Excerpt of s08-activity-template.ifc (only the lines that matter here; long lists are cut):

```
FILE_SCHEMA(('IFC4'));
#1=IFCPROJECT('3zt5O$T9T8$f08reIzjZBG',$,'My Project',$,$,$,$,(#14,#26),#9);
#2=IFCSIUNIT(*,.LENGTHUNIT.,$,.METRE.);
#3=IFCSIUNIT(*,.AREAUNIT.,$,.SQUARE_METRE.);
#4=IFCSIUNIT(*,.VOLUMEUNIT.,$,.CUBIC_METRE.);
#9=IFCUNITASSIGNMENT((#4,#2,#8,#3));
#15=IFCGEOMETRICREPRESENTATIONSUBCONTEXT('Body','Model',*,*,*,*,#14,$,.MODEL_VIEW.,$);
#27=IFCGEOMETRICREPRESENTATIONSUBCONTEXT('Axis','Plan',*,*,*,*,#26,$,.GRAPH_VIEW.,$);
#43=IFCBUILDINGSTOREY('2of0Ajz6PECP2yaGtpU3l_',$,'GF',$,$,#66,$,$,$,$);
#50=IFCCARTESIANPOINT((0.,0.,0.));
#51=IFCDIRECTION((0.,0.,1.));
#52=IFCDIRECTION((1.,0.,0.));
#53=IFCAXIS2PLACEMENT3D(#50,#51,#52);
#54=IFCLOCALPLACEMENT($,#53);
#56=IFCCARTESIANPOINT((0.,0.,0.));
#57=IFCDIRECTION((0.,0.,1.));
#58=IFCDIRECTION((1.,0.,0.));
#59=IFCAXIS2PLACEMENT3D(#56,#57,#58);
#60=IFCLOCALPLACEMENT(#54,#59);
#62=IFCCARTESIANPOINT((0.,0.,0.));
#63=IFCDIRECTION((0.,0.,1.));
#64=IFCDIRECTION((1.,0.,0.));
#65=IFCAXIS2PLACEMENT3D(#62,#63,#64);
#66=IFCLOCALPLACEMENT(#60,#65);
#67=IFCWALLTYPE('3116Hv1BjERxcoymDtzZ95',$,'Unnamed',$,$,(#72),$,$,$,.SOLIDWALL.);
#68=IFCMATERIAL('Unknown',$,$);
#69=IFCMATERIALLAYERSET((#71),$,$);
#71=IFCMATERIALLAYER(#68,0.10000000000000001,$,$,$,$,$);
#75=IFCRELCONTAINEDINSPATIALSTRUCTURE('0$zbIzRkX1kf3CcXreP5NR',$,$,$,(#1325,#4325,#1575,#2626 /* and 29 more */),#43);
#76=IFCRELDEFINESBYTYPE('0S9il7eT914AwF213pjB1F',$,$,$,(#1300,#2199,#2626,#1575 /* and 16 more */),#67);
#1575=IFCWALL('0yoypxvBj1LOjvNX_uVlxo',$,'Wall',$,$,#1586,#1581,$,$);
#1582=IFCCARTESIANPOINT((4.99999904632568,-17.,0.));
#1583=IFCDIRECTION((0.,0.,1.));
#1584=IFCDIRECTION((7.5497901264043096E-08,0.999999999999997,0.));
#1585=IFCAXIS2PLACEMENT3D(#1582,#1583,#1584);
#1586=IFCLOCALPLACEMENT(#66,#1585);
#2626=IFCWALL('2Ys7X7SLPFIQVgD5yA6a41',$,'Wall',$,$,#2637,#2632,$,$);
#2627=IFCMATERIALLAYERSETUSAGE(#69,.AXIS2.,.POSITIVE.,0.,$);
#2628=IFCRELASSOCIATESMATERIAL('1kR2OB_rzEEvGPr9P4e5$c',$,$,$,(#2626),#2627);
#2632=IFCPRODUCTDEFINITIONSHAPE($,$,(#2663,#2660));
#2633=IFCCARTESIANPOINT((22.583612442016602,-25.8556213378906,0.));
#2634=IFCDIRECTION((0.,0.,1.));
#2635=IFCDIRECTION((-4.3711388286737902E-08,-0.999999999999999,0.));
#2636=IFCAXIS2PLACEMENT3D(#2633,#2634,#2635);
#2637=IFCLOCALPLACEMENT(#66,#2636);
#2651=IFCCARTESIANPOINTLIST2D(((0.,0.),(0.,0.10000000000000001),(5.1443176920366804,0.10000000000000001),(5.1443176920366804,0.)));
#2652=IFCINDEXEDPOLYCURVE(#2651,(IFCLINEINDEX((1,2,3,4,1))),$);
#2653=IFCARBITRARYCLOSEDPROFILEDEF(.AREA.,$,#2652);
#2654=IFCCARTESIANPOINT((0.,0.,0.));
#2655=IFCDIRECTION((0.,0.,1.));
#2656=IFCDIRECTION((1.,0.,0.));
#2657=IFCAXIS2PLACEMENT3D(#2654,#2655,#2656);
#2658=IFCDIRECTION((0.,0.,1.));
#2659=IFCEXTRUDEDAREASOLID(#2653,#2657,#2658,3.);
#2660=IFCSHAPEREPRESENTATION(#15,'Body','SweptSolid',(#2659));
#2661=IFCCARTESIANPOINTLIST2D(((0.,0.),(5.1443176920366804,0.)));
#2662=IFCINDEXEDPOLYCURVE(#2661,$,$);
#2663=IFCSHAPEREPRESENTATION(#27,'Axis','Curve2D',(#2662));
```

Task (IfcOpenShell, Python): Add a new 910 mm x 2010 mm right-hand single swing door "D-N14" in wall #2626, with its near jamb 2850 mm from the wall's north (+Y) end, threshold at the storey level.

```python
import numpy as np
import ifcopenshell
import ifcopenshell.api.feature
import ifcopenshell.api.geometry
import ifcopenshell.api.root
import ifcopenshell.api.spatial
import ifcopenshell.geom
import ifcopenshell.util.element
import ifcopenshell.util.placement
import ifcopenshell.util.representation
import ifcopenshell.util.shape
import ifcopenshell.util.unit

model = ifcopenshell.open("s08-activity-template.ifc")
unit_scale = ifcopenshell.util.unit.calculate_unit_scale(model)
settings = ifcopenshell.geom.settings()


def volume(element):
    """Net volume in cubic metres, openings subtracted."""
    shape = ifcopenshell.geom.create_shape(settings, element)
    return ifcopenshell.util.shape.get_volume(shape.geometry)


wall = model.by_guid("2Ys7X7SLPFIQVgD5yA6a41")
storey = ifcopenshell.util.element.get_container(wall, ifc_class="IfcBuildingStorey")
context = ifcopenshell.util.representation.get_context(model, "Model", "Body", "MODEL_VIEW")
before = volume(wall)

width, height, from_end, sill = 0.91, 2.01, 2.85, 0.0  # metres

# The wall runs along its own X axis, and the end named is its -X end.
wall_shape = ifcopenshell.geom.create_shape(settings, wall)
x, y, z = ifcopenshell.util.shape.get_vertices(wall_shape.geometry).T
start = x.min() + from_end
face, thickness = float(y.min()), float(y.max() - y.min())
wall_matrix = ifcopenshell.util.placement.get_local_placement(wall.ObjectPlacement)
level = ifcopenshell.util.placement.get_local_placement(storey.ObjectPlacement)[2, 3]


def in_wall(x, y):
    """Placement at x, y metres in the wall's axes, at sill height."""
    matrix = wall_matrix.copy()
    matrix[:, 3] = wall_matrix @ np.array([x / unit_scale, y / unit_scale, 0.0, 1.0])
    matrix[2, 3] = level + sill / unit_scale
    return matrix


# Opening: a box that overshoots both wall faces by 50 mm.
opening = ifcopenshell.api.root.create_entity(model, ifc_class="IfcOpeningElement", predefined_type="OPENING")
box = ifcopenshell.api.geometry.add_wall_representation(
    model, context=context, length=width, height=height, thickness=thickness + 0.1
)
ifcopenshell.api.geometry.assign_representation(model, product=opening, representation=box)
ifcopenshell.api.geometry.edit_object_placement(model, product=opening, matrix=in_wall(start, face - 0.05), is_si=False)
ifcopenshell.api.feature.add_feature(model, feature=opening, element=wall)

door = ifcopenshell.api.root.create_entity(model, ifc_class="IfcDoor", name="D-N14", predefined_type="DOOR")
door.OverallWidth, door.OverallHeight = width / unit_scale, height / unit_scale
door.OperationType = "SINGLE_SWING_RIGHT"
body = ifcopenshell.api.geometry.add_door_representation(
    model,
    context=context,
    overall_width=door.OverallWidth,
    overall_height=door.OverallHeight,
    operation_type="SINGLE_SWING_RIGHT",
    lining_properties={"LiningDepth": thickness / unit_scale, "ThresholdDepth": thickness / unit_scale},
)
ifcopenshell.api.geometry.assign_representation(model, product=door, representation=body)
ifcopenshell.api.spatial.assign_container(model, products=[door], relating_structure=storey)
ifcopenshell.api.feature.add_filling(model, opening=opening, element=door)

# The lining spans the wall, so the door starts at the wall face.
ifcopenshell.api.geometry.edit_object_placement(model, product=door, matrix=in_wall(start, face), is_si=False)

after = volume(wall)

print(f"wall volume {before:.3f} -> {after:.3f} m3")

model.write("s08-activity-template_rev.ifc")
```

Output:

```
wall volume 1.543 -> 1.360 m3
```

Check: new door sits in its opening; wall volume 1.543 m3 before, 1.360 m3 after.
